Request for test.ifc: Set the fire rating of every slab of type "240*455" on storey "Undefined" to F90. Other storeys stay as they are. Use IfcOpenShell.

First a look at what the model holds.

```python
import ifcopenshell
import ifcopenshell.util.element

model = ifcopenshell.open("test.ifc")
print(model.schema)
storey = next(s for s in model.by_type("IfcBuildingStorey") if s.Name == "Undefined")
slabs = [e for e in ifcopenshell.util.element.get_decomposition(storey) if e.is_a("IfcSlab")]
seen = {}
for e in slabs:
    element_type = ifcopenshell.util.element.get_type(e)
    key = (element_type.Name if element_type != e and element_type else None, ifcopenshell.util.element.get_pset(e, "Pset_SlabCommon", "FireRating"))
    seen[key] = seen.get(key, 0) + 1
for (name, value), count in sorted(seen.items(), key=str):
    print(count, "x", name, "|", value)
```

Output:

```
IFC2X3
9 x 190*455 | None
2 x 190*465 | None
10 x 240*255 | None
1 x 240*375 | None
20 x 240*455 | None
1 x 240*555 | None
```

```python
import ifcopenshell
import ifcopenshell.api.pset
import ifcopenshell.util.element

model = ifcopenshell.open("test.ifc")

storey = next(s for s in model.by_type("IfcBuildingStorey") if s.Name == "Undefined")
slabs = [e for e in ifcopenshell.util.element.get_decomposition(storey) if e.is_a("IfcSlab")]

count = 0
for e in slabs:
    element_type = ifcopenshell.util.element.get_type(e)
    if element_type in (None, e) or element_type.Name != "240*455":
        continue
    found = ifcopenshell.util.element.get_pset(e, "Pset_SlabCommon", should_inherit=False)
    if found:
        pset = model.by_id(found["id"])
        if len(ifcopenshell.util.element.get_elements_by_pset(pset)) > 1:
            pset = ifcopenshell.api.pset.unshare_pset(model, products=[e], pset=pset)[0]
    else:
        pset = ifcopenshell.api.pset.add_pset(model, product=e, name="Pset_SlabCommon")
    ifcopenshell.api.pset.edit_pset(model, pset=pset, properties={"FireRating": "F90"})
    count += 1

print(count, "slabs updated")

model.write("test_updated.ifc")
```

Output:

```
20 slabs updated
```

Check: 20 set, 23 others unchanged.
